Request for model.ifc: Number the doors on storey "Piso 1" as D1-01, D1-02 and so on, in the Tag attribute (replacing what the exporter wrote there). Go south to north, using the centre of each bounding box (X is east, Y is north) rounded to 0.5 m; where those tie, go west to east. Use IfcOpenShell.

First a look at what the model holds.

```python
import ifcopenshell
import ifcopenshell.util.element
import ifcopenshell.util.placement

model = ifcopenshell.open("model.ifc")
print(model.schema)
storey = next(s for s in model.by_type("IfcBuildingStorey") if s.Name == "Piso 1")
doors = [e for e in ifcopenshell.util.element.get_decomposition(storey) if e.is_a("IfcDoor")]
for e in sorted(doors, key=lambda e: e.id()):
    origin = ifcopenshell.util.placement.get_local_placement(e.ObjectPlacement)[:3, 3]
    print(e.id(), e.Tag, e.Name, origin.round(2) + 0.0, sep=" | ")
```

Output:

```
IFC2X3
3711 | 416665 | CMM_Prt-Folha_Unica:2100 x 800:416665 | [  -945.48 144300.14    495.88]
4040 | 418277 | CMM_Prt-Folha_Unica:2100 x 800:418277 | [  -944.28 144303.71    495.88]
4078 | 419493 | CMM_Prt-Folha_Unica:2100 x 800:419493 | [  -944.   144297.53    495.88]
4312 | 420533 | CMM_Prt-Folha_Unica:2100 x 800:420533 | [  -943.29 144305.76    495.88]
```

```python
import ifcopenshell
import ifcopenshell.geom
import ifcopenshell.util.element
import ifcopenshell.util.shape

model = ifcopenshell.open("model.ifc")
settings = ifcopenshell.geom.settings()
settings.set("use-world-coords", True)


def centre(element):
    shape = ifcopenshell.geom.create_shape(settings, element)
    return ifcopenshell.util.shape.get_bbox_centroid(shape.geometry)


storey = next(s for s in model.by_type("IfcBuildingStorey") if s.Name == "Piso 1")
doors = [e for e in ifcopenshell.util.element.get_decomposition(storey) if e.is_a("IfcDoor")]

# Insertion points can sit at a corner or the storey origin, so sort by the geometry (in metres).
centres = {e: centre(e) for e in doors}
doors.sort(key=lambda e: (round(centres[e][1] / 0.5), centres[e][0]))

for i, e in enumerate(doors, start=1):
    number = f"D1-{i:02d}"
    e.Tag = number
    print(e.id(), number)

model.write("model_edited.ifc")
```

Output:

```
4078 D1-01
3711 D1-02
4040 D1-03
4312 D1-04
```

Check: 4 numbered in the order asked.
